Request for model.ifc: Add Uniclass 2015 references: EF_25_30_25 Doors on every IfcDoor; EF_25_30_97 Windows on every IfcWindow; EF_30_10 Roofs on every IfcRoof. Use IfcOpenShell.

First a look at what the model holds.

```python
import ifcopenshell

model = ifcopenshell.open("model.ifc")
print(model.schema)
print("classifications:", [c.Name for c in model.by_type("IfcClassification")])
for ifc_class in ("IfcDoor", "IfcRoof", "IfcStair", "IfcWall", "IfcWindow"):
    print(ifc_class, len(model.by_type(ifc_class)))
```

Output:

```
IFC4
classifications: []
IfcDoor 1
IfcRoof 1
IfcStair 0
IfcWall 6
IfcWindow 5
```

```python
import ifcopenshell
import ifcopenshell.api.classification

model = ifcopenshell.open("model.ifc")

system = ifcopenshell.api.classification.add_classification(model, classification="Uniclass 2015")

codes = {
    "IfcDoor": ("EF_25_30_25", "Doors"),
    "IfcWindow": ("EF_25_30_97", "Windows"),
    "IfcRoof": ("EF_30_10", "Roofs"),
}
for ifc_class, (code, name) in codes.items():
    products = model.by_type(ifc_class)
    ifcopenshell.api.classification.add_reference(
        model, products=products, classification=system, identification=code, name=name
    )
    print(code, len(products))

model.write("model_rev.ifc")
```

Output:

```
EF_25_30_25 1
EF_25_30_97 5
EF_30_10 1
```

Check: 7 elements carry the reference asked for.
